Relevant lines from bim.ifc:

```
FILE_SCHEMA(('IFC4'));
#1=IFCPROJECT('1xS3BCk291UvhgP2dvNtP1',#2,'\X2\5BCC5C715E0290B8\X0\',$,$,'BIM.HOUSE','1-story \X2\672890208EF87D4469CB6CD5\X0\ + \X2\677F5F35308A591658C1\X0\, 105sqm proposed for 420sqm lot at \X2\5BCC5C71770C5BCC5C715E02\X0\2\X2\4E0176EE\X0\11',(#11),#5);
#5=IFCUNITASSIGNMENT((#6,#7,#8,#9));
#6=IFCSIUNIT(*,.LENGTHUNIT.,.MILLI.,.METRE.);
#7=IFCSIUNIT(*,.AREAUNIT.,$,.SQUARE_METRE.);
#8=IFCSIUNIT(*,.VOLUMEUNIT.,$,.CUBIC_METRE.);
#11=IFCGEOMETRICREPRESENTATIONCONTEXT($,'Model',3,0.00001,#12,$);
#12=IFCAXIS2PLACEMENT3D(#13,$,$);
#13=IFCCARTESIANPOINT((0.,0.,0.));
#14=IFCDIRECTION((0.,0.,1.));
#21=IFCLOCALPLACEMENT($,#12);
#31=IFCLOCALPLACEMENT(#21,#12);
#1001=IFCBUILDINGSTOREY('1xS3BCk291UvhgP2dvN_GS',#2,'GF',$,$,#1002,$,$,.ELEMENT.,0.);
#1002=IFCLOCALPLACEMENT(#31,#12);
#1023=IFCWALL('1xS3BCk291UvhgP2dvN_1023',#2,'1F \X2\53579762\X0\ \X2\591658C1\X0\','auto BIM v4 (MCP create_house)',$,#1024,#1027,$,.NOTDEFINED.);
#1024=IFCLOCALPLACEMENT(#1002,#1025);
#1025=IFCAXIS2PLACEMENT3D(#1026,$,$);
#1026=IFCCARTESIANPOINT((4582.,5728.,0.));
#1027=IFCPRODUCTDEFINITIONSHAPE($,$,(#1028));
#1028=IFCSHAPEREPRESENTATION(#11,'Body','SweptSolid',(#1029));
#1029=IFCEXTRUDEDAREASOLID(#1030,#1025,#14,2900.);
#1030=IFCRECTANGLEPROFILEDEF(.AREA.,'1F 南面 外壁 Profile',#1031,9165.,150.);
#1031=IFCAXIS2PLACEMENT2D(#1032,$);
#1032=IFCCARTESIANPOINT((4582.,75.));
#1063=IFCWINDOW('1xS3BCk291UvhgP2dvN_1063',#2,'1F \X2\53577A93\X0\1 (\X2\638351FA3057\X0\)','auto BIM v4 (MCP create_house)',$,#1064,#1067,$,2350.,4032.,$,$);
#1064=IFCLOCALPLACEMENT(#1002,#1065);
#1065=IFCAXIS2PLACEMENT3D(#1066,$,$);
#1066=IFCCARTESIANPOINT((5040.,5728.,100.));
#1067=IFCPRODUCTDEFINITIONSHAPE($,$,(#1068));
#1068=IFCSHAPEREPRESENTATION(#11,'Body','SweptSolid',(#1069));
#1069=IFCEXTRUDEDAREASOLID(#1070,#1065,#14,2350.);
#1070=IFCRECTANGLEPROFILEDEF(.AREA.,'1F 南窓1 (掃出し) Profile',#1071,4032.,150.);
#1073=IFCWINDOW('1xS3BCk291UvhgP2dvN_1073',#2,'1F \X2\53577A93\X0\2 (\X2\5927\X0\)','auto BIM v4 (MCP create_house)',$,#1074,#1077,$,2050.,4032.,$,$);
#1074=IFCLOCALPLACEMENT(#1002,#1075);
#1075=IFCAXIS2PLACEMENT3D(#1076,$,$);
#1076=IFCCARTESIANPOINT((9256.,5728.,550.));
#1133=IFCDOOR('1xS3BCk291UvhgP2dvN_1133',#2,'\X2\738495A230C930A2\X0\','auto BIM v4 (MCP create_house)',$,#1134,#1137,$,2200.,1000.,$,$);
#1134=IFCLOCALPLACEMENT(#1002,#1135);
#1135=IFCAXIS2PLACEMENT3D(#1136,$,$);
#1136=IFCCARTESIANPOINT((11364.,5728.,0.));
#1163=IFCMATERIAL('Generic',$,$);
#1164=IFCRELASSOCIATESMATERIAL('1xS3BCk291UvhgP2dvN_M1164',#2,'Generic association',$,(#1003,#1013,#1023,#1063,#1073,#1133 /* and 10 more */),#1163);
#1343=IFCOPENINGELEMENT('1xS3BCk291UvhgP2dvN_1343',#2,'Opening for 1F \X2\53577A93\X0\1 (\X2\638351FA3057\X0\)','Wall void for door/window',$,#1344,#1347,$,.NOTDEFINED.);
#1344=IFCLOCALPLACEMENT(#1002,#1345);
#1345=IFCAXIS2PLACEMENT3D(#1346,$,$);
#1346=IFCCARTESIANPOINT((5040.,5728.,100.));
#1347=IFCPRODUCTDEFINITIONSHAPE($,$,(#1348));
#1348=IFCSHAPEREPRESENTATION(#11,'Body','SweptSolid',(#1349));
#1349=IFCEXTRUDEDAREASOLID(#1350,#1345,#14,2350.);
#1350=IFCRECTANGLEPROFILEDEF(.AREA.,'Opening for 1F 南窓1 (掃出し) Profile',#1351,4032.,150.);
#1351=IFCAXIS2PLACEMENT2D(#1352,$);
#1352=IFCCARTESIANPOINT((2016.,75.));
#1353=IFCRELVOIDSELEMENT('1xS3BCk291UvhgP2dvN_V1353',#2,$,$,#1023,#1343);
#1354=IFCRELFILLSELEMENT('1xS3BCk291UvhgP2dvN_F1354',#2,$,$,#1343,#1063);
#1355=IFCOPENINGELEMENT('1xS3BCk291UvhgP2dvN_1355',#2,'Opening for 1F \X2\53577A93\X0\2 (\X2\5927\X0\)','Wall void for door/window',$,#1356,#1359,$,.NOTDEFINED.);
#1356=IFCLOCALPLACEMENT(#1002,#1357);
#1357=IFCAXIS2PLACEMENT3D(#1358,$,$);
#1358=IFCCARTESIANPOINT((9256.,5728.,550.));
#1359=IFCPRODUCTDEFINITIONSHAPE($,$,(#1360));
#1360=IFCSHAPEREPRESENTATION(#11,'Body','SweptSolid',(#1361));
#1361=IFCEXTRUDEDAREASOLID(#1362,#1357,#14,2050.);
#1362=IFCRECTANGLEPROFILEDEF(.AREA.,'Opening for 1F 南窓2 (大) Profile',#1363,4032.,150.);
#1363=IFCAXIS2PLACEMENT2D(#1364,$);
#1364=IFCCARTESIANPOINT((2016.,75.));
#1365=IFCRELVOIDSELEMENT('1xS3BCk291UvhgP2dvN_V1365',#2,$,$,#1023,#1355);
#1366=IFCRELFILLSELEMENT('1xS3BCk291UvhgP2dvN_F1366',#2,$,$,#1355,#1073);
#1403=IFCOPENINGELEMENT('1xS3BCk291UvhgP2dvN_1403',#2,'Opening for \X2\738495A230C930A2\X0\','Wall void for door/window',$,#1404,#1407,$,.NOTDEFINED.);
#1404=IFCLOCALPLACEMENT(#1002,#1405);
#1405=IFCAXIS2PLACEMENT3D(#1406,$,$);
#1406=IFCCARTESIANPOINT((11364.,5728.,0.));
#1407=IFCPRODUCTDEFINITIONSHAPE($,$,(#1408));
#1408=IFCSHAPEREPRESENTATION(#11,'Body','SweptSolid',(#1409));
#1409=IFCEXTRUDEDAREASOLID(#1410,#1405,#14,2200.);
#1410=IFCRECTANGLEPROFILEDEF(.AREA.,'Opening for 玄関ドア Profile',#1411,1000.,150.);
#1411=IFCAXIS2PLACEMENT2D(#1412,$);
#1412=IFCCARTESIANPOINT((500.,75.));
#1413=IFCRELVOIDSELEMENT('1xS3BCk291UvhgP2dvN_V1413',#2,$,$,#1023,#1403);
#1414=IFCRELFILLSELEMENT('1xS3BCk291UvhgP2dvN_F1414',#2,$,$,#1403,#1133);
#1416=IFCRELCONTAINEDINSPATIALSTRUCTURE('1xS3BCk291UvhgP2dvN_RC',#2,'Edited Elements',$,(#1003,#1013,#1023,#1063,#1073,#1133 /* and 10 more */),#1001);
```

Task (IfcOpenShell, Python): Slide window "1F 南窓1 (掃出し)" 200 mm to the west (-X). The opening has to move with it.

```python
import ifcopenshell
import ifcopenshell.api.geometry
import ifcopenshell.util.placement
import ifcopenshell.util.unit

model = ifcopenshell.open("bim.ifc")
unit_scale = ifcopenshell.util.unit.calculate_unit_scale(model)

window = model.by_id(1063)
opening = window.FillsVoids[0].RelatingOpeningElement
wall = opening.VoidsElements[0].RelatingBuildingElement

wall_matrix = ifcopenshell.util.placement.get_local_placement(wall.ObjectPlacement)
shift = wall_matrix[:3, 0] * -0.2 / unit_scale
before = ifcopenshell.util.placement.get_local_placement(window.ObjectPlacement)[:3, 3].copy()

# The window is not placed relative to its opening, so move both.
for product in (opening, window):
    matrix = ifcopenshell.util.placement.get_local_placement(product.ObjectPlacement)
    matrix[:3, 3] += shift
    ifcopenshell.api.geometry.edit_object_placement(model, product=product, matrix=matrix, is_si=False)

after = ifcopenshell.util.placement.get_local_placement(window.ObjectPlacement)[:3, 3]
print("window moved by", (after - before).round(3) + 0.0)

model.write("bim_edited.ifc")
```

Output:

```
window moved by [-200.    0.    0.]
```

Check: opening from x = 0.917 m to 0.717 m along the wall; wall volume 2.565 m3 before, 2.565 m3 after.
